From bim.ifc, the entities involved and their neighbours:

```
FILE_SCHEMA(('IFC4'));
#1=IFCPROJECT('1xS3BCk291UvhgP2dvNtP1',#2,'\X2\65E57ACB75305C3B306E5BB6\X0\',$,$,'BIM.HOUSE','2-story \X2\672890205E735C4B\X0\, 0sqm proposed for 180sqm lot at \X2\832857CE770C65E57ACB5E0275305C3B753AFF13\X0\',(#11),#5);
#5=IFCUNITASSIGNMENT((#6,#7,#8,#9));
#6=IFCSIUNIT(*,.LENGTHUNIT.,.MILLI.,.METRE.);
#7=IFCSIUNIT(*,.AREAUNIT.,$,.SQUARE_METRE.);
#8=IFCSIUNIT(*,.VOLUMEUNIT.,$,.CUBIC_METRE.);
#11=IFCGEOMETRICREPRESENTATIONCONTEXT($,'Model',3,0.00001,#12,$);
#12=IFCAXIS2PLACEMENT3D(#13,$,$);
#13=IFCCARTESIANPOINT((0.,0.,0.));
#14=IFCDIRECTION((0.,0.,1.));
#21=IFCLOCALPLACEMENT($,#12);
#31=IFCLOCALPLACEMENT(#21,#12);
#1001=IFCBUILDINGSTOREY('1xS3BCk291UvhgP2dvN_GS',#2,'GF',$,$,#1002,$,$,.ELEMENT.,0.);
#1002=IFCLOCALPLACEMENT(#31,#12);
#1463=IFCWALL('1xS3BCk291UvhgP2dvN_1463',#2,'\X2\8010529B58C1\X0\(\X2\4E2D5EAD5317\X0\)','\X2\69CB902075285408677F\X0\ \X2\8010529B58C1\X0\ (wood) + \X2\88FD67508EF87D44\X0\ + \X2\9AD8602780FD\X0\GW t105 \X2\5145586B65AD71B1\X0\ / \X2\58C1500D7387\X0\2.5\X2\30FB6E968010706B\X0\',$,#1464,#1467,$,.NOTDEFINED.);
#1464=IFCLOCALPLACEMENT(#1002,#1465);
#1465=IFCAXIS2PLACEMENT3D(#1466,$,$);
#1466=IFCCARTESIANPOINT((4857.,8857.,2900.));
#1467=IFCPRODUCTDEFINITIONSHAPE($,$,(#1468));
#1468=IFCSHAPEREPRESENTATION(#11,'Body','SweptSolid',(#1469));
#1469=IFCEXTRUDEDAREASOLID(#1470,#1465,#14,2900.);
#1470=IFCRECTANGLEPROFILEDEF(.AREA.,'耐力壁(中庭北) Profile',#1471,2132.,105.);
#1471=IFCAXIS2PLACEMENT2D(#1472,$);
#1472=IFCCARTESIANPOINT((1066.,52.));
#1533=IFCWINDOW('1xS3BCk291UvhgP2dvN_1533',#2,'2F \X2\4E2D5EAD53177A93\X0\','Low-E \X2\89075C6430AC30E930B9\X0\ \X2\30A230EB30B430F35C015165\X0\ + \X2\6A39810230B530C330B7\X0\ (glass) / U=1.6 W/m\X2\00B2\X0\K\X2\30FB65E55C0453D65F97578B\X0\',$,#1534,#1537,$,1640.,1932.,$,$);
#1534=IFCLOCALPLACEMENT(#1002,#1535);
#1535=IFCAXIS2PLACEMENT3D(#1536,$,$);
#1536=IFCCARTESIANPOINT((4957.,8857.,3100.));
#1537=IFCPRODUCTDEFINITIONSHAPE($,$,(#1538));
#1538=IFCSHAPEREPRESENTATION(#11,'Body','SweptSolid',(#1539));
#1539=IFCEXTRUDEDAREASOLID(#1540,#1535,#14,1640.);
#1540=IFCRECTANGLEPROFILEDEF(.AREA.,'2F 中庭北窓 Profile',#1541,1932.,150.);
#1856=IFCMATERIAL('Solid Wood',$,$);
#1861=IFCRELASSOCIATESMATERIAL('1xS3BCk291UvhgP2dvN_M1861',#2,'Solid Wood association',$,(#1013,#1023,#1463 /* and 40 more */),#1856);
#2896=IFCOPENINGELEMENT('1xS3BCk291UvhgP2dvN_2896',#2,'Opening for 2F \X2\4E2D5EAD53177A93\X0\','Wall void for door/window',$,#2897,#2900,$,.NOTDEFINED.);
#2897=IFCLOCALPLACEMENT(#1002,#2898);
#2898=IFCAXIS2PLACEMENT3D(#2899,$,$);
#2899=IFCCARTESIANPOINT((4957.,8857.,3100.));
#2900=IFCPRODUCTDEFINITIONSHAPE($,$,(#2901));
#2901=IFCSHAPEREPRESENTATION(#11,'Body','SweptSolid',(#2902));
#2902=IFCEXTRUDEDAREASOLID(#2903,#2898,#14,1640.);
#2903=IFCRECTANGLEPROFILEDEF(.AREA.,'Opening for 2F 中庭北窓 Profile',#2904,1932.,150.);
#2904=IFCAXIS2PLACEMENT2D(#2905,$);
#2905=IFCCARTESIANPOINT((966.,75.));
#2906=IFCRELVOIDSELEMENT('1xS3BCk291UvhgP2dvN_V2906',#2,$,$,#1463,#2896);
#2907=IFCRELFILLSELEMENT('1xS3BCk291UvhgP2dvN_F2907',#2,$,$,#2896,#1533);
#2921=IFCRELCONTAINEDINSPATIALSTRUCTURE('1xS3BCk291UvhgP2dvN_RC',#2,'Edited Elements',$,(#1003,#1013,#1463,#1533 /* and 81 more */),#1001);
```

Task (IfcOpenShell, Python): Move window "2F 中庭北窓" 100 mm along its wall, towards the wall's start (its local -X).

```python
import ifcopenshell
import ifcopenshell.api.geometry
import ifcopenshell.util.placement
import ifcopenshell.util.unit

model = ifcopenshell.open("bim.ifc")
unit_scale = ifcopenshell.util.unit.calculate_unit_scale(model)

window = model.by_id(1533)
opening = window.FillsVoids[0].RelatingOpeningElement
wall = opening.VoidsElements[0].RelatingBuildingElement

wall_matrix = ifcopenshell.util.placement.get_local_placement(wall.ObjectPlacement)
shift = wall_matrix[:3, 0] * -0.1 / unit_scale
before = ifcopenshell.util.placement.get_local_placement(window.ObjectPlacement)[:3, 3].copy()

# The window is not placed relative to its opening, so move both.
for product in (opening, window):
    matrix = ifcopenshell.util.placement.get_local_placement(product.ObjectPlacement)
    matrix[:3, 3] += shift
    ifcopenshell.api.geometry.edit_object_placement(model, product=product, matrix=matrix, is_si=False)

after = ifcopenshell.util.placement.get_local_placement(window.ObjectPlacement)[:3, 3]
print("window moved by", (after - before).round(3) + 0.0)

model.write("bim_rev.ifc")
```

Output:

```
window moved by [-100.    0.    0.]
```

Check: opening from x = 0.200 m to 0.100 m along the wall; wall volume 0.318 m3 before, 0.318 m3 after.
